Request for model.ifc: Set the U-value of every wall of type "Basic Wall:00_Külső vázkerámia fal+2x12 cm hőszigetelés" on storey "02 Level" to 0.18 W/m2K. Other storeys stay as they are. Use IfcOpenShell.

First a look at what the model holds.

```python
import ifcopenshell
import ifcopenshell.util.element

model = ifcopenshell.open("model.ifc")
print(model.schema)
storey = next(s for s in model.by_type("IfcBuildingStorey") if s.Name == "02 Level")
walls = [e for e in ifcopenshell.util.element.get_decomposition(storey) if e.is_a("IfcWall")]
seen = {}
for e in walls:
    element_type = ifcopenshell.util.element.get_type(e)
    key = (element_type.Name if element_type != e and element_type else None, ifcopenshell.util.element.get_pset(e, "Pset_WallCommon", "ThermalTransmittance"))
    seen[key] = seen.get(key, 0) + 1
for (name, value), count in sorted(seen.items(), key=str):
    print(count, "x", name, "|", value)
```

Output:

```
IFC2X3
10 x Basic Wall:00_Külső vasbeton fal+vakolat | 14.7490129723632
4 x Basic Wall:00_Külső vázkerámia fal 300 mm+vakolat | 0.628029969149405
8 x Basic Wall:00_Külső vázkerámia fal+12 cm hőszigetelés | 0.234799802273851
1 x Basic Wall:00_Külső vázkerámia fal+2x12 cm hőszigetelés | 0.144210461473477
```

```python
import ifcopenshell
import ifcopenshell.api.pset
import ifcopenshell.util.element

model = ifcopenshell.open("model.ifc")

storey = next(s for s in model.by_type("IfcBuildingStorey") if s.Name == "02 Level")
walls = [e for e in ifcopenshell.util.element.get_decomposition(storey) if e.is_a("IfcWall")]

count = 0
for e in walls:
    element_type = ifcopenshell.util.element.get_type(e)
    if element_type in (None, e) or element_type.Name != "Basic Wall:00_Külső vázkerámia fal+2x12 cm hőszigetelés":
        continue
    # add_pset returns the element's existing set when there is one.
    pset = ifcopenshell.api.pset.add_pset(model, product=e, name="Pset_WallCommon")
    ifcopenshell.api.pset.edit_pset(model, pset=pset, properties={"ThermalTransmittance": 0.18})
    count += 1

print(count, "walls updated")

model.write("model-out.ifc")
```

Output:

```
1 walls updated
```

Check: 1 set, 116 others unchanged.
